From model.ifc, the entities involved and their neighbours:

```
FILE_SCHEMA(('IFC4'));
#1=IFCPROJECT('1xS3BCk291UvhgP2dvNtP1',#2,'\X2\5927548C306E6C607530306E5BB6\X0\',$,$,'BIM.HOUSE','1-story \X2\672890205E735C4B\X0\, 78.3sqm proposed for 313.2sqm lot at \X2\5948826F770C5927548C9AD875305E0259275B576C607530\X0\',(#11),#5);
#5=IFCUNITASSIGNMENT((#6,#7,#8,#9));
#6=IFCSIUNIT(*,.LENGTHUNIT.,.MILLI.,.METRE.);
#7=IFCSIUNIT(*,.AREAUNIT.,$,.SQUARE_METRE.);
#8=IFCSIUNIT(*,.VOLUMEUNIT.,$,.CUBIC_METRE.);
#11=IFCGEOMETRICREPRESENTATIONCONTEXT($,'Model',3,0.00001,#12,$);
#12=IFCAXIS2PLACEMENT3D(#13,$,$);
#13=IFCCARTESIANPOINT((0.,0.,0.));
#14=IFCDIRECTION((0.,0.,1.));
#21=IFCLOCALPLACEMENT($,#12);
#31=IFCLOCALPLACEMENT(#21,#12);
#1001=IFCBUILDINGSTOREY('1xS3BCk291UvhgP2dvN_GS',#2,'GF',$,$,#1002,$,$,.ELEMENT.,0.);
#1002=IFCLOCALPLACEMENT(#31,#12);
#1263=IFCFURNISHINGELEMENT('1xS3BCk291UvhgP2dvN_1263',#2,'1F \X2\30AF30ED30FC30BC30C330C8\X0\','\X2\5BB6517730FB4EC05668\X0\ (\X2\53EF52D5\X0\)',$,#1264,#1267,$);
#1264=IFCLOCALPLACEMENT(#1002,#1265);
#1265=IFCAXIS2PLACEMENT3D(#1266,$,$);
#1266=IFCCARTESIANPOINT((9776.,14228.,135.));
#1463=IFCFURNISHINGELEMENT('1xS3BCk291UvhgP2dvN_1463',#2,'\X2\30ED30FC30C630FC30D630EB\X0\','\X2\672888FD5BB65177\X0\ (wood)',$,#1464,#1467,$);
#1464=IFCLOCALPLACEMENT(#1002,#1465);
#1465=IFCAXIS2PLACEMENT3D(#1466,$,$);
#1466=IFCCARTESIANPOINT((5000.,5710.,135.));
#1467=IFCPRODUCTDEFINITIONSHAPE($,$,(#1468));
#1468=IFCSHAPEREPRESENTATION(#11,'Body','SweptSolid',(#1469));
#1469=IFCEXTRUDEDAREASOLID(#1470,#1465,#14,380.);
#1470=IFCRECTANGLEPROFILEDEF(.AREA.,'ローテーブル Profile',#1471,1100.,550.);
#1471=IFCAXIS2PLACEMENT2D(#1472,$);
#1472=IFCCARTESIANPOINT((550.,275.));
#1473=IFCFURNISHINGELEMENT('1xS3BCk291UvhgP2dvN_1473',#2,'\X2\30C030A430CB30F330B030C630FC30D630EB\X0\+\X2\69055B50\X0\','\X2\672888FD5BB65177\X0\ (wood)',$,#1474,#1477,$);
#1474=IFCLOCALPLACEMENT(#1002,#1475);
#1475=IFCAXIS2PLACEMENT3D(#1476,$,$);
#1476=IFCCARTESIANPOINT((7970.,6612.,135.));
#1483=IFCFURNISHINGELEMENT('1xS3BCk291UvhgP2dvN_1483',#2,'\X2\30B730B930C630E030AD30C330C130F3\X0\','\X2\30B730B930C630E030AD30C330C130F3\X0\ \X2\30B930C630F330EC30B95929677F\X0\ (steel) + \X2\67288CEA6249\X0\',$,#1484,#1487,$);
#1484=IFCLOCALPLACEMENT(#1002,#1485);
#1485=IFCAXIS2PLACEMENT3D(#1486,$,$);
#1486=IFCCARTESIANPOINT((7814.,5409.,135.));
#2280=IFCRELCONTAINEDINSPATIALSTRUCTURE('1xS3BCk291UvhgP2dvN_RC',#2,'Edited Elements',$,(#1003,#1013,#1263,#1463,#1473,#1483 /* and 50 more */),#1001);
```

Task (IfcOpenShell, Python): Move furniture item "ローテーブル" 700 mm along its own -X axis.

```python
import ifcopenshell
import ifcopenshell.api.geometry
import ifcopenshell.util.placement
import ifcopenshell.util.unit

model = ifcopenshell.open("model.ifc")
unit_scale = ifcopenshell.util.unit.calculate_unit_scale(model)

item = model.by_guid("1xS3BCk291UvhgP2dvN_1463")
matrix = ifcopenshell.util.placement.get_local_placement(item.ObjectPlacement)
matrix[:3, 3] -= matrix[:3, 0] * 0.7 / unit_scale
ifcopenshell.api.geometry.edit_object_placement(model, product=item, matrix=matrix, is_si=False)

print(ifcopenshell.util.placement.get_local_placement(item.ObjectPlacement).round(3) + 0.0)

model.write("model-out.ifc")
```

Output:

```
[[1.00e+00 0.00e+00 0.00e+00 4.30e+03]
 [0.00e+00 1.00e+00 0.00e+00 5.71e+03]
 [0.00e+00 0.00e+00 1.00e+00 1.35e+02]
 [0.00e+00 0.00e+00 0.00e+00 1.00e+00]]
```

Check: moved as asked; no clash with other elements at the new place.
